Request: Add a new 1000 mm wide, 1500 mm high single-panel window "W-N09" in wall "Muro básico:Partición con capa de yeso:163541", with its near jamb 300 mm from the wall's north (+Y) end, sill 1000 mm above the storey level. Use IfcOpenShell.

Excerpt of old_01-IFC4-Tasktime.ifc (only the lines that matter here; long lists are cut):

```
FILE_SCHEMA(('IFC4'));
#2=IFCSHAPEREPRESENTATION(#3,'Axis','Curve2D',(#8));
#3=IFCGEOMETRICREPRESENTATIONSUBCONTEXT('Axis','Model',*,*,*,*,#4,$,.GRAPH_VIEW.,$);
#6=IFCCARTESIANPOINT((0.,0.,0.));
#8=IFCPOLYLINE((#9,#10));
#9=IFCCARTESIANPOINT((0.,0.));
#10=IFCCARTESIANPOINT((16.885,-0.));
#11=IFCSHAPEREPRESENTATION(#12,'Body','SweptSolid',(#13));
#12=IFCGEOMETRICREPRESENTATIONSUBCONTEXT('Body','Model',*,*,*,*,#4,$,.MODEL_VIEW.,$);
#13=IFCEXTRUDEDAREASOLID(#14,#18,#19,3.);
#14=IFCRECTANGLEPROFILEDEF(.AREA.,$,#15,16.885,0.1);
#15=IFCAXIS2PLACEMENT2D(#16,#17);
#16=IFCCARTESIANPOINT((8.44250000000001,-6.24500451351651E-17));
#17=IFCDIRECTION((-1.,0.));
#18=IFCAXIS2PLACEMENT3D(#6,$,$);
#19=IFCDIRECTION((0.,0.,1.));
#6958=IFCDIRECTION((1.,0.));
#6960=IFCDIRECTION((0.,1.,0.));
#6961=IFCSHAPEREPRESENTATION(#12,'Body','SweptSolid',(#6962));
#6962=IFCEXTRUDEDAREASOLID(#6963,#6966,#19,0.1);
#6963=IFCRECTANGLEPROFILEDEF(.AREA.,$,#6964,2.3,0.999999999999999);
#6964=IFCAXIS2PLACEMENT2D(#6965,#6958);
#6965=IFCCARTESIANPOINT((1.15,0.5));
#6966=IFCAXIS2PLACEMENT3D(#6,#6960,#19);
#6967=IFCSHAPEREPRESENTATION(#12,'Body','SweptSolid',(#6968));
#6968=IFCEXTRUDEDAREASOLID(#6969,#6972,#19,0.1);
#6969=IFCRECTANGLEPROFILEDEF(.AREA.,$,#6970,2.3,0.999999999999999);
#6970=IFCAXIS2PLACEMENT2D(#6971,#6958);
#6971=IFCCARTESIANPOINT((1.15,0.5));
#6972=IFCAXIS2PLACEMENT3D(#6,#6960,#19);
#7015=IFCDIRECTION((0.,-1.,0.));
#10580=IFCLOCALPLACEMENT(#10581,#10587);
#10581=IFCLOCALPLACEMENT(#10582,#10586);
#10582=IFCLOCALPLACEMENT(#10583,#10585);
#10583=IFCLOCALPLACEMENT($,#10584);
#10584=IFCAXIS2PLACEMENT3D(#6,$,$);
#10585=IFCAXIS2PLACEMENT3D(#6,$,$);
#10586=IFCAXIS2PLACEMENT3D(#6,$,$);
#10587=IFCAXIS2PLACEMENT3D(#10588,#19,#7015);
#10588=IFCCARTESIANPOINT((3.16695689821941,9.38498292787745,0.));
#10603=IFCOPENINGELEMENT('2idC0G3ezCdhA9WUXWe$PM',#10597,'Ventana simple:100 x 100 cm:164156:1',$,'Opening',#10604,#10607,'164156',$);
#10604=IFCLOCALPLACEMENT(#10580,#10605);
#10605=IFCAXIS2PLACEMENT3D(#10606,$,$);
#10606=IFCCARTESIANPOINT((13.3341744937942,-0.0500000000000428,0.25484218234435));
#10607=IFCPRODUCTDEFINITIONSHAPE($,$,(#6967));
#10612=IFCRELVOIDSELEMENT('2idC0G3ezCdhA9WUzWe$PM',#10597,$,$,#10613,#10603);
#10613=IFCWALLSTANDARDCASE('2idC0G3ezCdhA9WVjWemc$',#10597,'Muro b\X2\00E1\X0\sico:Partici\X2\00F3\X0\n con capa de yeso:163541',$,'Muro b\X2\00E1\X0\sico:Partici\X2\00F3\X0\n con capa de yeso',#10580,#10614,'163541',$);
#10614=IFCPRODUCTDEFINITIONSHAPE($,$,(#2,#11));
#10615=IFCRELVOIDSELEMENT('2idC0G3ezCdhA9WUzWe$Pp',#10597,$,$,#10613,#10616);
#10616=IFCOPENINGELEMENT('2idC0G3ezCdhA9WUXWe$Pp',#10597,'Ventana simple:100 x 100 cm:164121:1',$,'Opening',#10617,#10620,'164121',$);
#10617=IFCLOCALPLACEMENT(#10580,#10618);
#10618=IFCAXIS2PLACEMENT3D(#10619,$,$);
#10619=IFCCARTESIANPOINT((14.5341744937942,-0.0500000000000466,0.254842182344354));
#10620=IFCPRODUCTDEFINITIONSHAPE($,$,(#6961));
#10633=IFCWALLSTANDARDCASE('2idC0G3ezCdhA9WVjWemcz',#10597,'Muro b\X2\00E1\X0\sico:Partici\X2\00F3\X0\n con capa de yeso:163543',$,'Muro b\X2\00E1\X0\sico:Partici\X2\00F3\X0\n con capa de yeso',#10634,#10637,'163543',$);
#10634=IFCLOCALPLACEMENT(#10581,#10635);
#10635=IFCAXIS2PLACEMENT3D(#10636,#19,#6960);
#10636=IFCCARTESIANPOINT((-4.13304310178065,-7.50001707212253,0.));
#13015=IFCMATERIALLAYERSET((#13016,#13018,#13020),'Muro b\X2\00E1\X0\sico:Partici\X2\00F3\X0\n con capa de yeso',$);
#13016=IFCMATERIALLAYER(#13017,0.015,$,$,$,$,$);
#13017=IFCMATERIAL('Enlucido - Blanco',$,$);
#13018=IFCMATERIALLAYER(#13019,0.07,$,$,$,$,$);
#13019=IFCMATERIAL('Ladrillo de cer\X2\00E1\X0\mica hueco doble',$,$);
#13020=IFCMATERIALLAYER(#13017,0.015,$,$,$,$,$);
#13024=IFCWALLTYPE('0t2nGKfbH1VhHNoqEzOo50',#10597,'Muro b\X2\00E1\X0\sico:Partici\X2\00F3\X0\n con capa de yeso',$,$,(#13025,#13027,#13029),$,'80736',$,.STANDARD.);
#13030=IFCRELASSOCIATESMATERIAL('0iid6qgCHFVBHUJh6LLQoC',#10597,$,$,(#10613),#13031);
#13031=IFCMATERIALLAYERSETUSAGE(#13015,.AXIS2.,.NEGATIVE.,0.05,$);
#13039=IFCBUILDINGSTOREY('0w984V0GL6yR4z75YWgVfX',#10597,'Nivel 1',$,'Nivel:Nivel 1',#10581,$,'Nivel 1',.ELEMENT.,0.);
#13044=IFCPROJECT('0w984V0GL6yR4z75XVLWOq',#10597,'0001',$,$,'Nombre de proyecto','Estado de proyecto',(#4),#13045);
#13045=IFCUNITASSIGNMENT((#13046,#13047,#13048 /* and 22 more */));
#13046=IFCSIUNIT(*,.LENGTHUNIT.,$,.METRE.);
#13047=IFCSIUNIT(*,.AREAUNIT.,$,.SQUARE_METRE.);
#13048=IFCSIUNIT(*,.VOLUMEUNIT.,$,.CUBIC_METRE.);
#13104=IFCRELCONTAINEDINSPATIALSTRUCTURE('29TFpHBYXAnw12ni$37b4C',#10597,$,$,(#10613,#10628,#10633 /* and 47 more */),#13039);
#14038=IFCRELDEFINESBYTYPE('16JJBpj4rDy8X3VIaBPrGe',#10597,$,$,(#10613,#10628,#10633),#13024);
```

```python
import numpy as np
import ifcopenshell
import ifcopenshell.api.feature
import ifcopenshell.api.geometry
import ifcopenshell.api.root
import ifcopenshell.api.spatial
import ifcopenshell.geom
import ifcopenshell.util.element
import ifcopenshell.util.placement
import ifcopenshell.util.representation
import ifcopenshell.util.shape
import ifcopenshell.util.unit

model = ifcopenshell.open("old_01-IFC4-Tasktime.ifc")
unit_scale = ifcopenshell.util.unit.calculate_unit_scale(model)
settings = ifcopenshell.geom.settings()


def volume(element):
    """Net volume in cubic metres, openings subtracted."""
    shape = ifcopenshell.geom.create_shape(settings, element)
    return ifcopenshell.util.shape.get_volume(shape.geometry)


wall = model.by_id(10613)
storey = ifcopenshell.util.element.get_container(wall, ifc_class="IfcBuildingStorey")
context = ifcopenshell.util.representation.get_context(model, "Model", "Body", "MODEL_VIEW")
before = volume(wall)

width, height, from_end, sill = 1, 1.5, 0.3, 1  # metres

# The wall runs along its own X axis, and the end named is its -X end.
wall_shape = ifcopenshell.geom.create_shape(settings, wall)
x, y, z = ifcopenshell.util.shape.get_vertices(wall_shape.geometry).T
start = x.min() + from_end
face, thickness = float(y.min()), float(y.max() - y.min())
wall_matrix = ifcopenshell.util.placement.get_local_placement(wall.ObjectPlacement)
level = ifcopenshell.util.placement.get_local_placement(storey.ObjectPlacement)[2, 3]


def in_wall(x, y):
    """Placement at x, y metres in the wall's axes, at sill height."""
    matrix = wall_matrix.copy()
    matrix[:, 3] = wall_matrix @ np.array([x / unit_scale, y / unit_scale, 0.0, 1.0])
    matrix[2, 3] = level + sill / unit_scale
    return matrix


# Opening: a box that overshoots both wall faces by 50 mm.
opening = ifcopenshell.api.root.create_entity(model, ifc_class="IfcOpeningElement", predefined_type="OPENING")
box = ifcopenshell.api.geometry.add_wall_representation(
    model, context=context, length=width, height=height, thickness=thickness + 0.1
)
ifcopenshell.api.geometry.assign_representation(model, product=opening, representation=box)
ifcopenshell.api.geometry.edit_object_placement(model, product=opening, matrix=in_wall(start, face - 0.05), is_si=False)
ifcopenshell.api.feature.add_feature(model, feature=opening, element=wall)

window = ifcopenshell.api.root.create_entity(model, ifc_class="IfcWindow", name="W-N09", predefined_type="WINDOW")
window.OverallWidth, window.OverallHeight = width / unit_scale, height / unit_scale
window.PartitioningType = "SINGLE_PANEL"
body = ifcopenshell.api.geometry.add_window_representation(
    model,
    context=context,
    overall_width=window.OverallWidth,
    overall_height=window.OverallHeight,
    partition_type="SINGLE_PANEL",
)
ifcopenshell.api.geometry.assign_representation(model, product=window, representation=body)
ifcopenshell.api.spatial.assign_container(model, products=[window], relating_structure=storey)
ifcopenshell.api.feature.add_filling(model, opening=opening, element=window)

# Centre the window in the wall's thickness.
ifcopenshell.api.geometry.edit_object_placement(model, product=window, matrix=in_wall(start, face), is_si=False)
window_shape = ifcopenshell.geom.create_shape(settings, window)
depth = ifcopenshell.util.shape.get_vertices(window_shape.geometry)[:, 1]
offset = face + thickness / 2 - (depth.min() + depth.max()) / 2
ifcopenshell.api.geometry.edit_object_placement(model, product=window, matrix=in_wall(start, offset), is_si=False)

after = volume(wall)

print(f"wall volume {before:.3f} -> {after:.3f} m3")

model.write("old_01-IFC4-Tasktime-out.ifc")
```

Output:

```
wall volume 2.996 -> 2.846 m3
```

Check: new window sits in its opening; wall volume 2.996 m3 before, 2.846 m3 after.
